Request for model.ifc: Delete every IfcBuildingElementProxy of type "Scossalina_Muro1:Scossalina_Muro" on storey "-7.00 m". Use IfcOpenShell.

First a look at what the model holds.

```python
import ifcopenshell
import ifcopenshell.util.element

model = ifcopenshell.open("model.ifc")
print(model.schema)
storey = next(s for s in model.by_type("IfcBuildingStorey") if s.Name == "-7.00 m")
proxies = [e for e in ifcopenshell.util.element.get_decomposition(storey) if e.is_a("IfcBuildingElementProxy")]
seen = {}
for e in proxies:
    element_type = ifcopenshell.util.element.get_type(e)
    name = element_type.Name if element_type not in (None, e) else None
    seen[name] = seen.get(name, 0) + 1
for name, count in sorted(seen.items(), key=str):
    print(count, "x", name)
```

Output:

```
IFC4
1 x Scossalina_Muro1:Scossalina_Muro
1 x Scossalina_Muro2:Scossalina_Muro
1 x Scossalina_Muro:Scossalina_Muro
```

```python
import ifcopenshell
import ifcopenshell.api.root
import ifcopenshell.util.element

model = ifcopenshell.open("model.ifc")

storey = next(s for s in model.by_type("IfcBuildingStorey") if s.Name == "-7.00 m")
proxies = [e for e in ifcopenshell.util.element.get_decomposition(storey) if e.is_a("IfcBuildingElementProxy")]
targets = [e for e in proxies if (t := ifcopenshell.util.element.get_type(e)) not in (None, e) and t.Name == "Scossalina_Muro1:Scossalina_Muro"]

for e in targets:
    ifcopenshell.api.root.remove_product(model, product=e)
print(len(targets), "removed")

model.write("model_edited.ifc")
```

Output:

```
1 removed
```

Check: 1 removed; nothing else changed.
